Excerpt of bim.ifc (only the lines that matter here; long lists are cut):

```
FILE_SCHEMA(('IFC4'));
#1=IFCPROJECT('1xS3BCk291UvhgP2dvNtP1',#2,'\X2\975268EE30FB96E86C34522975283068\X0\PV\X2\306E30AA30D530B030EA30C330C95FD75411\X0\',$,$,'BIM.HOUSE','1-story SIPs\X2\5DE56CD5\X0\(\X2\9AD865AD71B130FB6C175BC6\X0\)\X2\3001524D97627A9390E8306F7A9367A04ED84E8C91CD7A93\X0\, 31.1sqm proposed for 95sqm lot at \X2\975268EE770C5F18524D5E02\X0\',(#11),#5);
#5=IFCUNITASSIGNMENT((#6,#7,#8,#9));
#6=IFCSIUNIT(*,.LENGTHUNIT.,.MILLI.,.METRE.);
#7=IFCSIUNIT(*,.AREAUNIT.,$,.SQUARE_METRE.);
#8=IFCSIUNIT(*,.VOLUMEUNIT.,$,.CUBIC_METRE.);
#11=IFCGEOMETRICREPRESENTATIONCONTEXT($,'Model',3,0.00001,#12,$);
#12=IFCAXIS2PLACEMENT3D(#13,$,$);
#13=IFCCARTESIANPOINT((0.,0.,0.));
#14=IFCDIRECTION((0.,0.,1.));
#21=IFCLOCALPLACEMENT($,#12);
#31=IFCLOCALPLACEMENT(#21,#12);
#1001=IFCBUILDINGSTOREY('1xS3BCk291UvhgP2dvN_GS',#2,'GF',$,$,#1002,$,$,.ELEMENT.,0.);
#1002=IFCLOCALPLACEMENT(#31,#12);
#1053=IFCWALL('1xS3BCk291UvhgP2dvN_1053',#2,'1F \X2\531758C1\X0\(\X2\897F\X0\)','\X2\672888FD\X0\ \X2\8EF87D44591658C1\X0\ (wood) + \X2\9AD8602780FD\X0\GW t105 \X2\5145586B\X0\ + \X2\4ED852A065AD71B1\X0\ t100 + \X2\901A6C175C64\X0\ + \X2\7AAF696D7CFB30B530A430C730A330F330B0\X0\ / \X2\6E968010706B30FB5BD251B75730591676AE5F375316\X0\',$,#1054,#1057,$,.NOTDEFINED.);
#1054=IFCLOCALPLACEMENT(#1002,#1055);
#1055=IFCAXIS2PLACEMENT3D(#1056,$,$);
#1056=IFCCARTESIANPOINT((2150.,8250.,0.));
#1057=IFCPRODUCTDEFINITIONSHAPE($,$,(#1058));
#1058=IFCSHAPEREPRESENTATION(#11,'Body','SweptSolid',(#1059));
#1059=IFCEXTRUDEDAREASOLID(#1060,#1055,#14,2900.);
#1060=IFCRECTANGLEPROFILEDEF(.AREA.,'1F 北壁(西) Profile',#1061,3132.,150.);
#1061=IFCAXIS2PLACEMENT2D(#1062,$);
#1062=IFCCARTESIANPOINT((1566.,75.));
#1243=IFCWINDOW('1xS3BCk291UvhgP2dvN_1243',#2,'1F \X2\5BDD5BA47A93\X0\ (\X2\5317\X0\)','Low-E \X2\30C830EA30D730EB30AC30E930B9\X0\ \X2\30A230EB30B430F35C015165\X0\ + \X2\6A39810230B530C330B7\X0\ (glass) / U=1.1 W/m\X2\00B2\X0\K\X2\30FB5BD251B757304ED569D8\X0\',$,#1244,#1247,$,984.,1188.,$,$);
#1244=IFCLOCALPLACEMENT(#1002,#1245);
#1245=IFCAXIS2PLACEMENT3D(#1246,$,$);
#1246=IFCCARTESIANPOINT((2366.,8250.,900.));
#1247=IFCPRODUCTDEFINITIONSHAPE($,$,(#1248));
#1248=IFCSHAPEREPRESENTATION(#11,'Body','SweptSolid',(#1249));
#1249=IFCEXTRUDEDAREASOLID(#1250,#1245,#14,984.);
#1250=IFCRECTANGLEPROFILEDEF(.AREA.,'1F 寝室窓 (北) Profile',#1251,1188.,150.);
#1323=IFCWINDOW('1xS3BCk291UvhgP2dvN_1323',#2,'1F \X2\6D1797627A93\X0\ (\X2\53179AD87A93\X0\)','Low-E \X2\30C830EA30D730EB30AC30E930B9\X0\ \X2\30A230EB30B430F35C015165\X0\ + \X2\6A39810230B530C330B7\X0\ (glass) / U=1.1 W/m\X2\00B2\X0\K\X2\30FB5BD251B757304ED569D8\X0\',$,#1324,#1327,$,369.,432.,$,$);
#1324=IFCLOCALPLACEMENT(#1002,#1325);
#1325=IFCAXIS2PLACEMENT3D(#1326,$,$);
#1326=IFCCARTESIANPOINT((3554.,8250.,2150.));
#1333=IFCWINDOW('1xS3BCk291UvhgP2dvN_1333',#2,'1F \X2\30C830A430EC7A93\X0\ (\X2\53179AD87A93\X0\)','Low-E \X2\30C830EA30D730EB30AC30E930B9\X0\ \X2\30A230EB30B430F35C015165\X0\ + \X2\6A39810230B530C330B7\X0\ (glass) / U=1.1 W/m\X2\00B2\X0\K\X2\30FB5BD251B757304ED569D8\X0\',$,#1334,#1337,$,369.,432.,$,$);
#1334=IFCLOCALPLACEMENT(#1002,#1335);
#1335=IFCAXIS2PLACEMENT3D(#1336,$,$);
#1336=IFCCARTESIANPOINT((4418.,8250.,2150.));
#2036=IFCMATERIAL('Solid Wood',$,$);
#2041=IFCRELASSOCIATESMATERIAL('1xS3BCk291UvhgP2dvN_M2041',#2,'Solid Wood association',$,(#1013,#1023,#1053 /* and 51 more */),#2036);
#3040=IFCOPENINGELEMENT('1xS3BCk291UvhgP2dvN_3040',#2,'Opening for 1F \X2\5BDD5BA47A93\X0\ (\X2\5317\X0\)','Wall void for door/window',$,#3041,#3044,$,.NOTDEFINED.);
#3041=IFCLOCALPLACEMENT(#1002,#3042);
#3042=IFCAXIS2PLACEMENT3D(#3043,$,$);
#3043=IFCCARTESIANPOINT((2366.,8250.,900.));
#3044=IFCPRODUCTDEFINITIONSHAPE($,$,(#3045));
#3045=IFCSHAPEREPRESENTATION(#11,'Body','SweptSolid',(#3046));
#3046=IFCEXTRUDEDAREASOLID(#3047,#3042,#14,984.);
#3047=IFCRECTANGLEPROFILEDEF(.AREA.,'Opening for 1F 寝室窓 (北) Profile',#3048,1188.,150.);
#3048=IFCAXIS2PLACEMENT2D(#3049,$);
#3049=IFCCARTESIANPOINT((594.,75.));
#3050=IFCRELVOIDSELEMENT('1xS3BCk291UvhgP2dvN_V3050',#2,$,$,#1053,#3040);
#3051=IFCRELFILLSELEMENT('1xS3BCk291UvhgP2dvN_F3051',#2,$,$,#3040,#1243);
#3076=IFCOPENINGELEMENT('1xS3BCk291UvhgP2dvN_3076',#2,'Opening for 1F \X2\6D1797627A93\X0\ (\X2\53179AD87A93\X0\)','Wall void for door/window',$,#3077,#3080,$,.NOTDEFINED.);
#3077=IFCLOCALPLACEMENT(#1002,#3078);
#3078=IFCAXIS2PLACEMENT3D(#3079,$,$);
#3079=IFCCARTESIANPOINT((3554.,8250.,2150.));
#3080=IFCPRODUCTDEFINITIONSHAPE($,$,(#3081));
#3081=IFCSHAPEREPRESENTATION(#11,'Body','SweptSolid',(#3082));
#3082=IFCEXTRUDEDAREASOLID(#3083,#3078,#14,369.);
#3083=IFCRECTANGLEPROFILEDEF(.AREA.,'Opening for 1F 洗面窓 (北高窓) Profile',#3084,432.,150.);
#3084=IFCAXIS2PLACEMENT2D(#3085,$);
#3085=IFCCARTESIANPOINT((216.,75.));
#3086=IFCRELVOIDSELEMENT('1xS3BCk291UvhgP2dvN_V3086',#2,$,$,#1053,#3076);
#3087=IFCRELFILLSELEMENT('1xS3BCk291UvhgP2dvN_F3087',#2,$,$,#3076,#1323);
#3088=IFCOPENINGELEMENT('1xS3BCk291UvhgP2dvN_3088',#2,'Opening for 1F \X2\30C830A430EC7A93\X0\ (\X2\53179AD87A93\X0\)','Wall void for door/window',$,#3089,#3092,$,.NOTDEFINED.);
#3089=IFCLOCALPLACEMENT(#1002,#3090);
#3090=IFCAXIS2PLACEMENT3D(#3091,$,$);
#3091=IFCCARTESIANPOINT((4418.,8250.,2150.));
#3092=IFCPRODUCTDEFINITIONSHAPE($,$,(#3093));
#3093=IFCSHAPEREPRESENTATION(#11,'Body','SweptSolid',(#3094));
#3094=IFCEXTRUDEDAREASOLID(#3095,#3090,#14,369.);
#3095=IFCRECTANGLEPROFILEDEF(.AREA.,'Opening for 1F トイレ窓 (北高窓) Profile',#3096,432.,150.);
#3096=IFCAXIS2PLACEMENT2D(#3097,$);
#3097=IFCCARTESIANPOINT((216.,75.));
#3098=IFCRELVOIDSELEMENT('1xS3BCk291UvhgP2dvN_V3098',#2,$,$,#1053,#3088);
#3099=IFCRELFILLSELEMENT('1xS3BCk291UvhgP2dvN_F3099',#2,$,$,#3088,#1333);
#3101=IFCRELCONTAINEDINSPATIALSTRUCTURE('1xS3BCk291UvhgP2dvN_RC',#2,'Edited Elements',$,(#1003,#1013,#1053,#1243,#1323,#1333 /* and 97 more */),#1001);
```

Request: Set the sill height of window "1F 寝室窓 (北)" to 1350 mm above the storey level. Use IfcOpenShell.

```python
import numpy as np
import ifcopenshell
import ifcopenshell.api.geometry
import ifcopenshell.geom
import ifcopenshell.util.element
import ifcopenshell.util.placement
import ifcopenshell.util.shape
import ifcopenshell.util.unit

model = ifcopenshell.open("bim.ifc")
unit_scale = ifcopenshell.util.unit.calculate_unit_scale(model)

window = model.by_guid("1xS3BCk291UvhgP2dvN_1243")
opening = window.FillsVoids[0].RelatingOpeningElement
storey = ifcopenshell.util.element.get_container(window, ifc_class="IfcBuildingStorey")
level = ifcopenshell.util.placement.get_local_placement(storey.ObjectPlacement)[2, 3]

# The opening's origin need not be at the sill, so measure its lowest point.
shape = ifcopenshell.geom.create_shape(ifcopenshell.geom.settings(), opening)
bottom = ifcopenshell.util.shape.get_shape_bottom_elevation(shape, shape.geometry) / unit_scale
dz = level + 1.35 / unit_scale - bottom

shift = np.array([0.0, 0.0, dz])
# The window is not placed relative to its opening, so move both.
for product in (opening, window):
    matrix = ifcopenshell.util.placement.get_local_placement(product.ObjectPlacement)
    matrix[:3, 3] += shift
    ifcopenshell.api.geometry.edit_object_placement(model, product=product, matrix=matrix, is_si=False)

print(f"moved by {dz * unit_scale:+.3f} m")

model.write("bim_updated.ifc")
```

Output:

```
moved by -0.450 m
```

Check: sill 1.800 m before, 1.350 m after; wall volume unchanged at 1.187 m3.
